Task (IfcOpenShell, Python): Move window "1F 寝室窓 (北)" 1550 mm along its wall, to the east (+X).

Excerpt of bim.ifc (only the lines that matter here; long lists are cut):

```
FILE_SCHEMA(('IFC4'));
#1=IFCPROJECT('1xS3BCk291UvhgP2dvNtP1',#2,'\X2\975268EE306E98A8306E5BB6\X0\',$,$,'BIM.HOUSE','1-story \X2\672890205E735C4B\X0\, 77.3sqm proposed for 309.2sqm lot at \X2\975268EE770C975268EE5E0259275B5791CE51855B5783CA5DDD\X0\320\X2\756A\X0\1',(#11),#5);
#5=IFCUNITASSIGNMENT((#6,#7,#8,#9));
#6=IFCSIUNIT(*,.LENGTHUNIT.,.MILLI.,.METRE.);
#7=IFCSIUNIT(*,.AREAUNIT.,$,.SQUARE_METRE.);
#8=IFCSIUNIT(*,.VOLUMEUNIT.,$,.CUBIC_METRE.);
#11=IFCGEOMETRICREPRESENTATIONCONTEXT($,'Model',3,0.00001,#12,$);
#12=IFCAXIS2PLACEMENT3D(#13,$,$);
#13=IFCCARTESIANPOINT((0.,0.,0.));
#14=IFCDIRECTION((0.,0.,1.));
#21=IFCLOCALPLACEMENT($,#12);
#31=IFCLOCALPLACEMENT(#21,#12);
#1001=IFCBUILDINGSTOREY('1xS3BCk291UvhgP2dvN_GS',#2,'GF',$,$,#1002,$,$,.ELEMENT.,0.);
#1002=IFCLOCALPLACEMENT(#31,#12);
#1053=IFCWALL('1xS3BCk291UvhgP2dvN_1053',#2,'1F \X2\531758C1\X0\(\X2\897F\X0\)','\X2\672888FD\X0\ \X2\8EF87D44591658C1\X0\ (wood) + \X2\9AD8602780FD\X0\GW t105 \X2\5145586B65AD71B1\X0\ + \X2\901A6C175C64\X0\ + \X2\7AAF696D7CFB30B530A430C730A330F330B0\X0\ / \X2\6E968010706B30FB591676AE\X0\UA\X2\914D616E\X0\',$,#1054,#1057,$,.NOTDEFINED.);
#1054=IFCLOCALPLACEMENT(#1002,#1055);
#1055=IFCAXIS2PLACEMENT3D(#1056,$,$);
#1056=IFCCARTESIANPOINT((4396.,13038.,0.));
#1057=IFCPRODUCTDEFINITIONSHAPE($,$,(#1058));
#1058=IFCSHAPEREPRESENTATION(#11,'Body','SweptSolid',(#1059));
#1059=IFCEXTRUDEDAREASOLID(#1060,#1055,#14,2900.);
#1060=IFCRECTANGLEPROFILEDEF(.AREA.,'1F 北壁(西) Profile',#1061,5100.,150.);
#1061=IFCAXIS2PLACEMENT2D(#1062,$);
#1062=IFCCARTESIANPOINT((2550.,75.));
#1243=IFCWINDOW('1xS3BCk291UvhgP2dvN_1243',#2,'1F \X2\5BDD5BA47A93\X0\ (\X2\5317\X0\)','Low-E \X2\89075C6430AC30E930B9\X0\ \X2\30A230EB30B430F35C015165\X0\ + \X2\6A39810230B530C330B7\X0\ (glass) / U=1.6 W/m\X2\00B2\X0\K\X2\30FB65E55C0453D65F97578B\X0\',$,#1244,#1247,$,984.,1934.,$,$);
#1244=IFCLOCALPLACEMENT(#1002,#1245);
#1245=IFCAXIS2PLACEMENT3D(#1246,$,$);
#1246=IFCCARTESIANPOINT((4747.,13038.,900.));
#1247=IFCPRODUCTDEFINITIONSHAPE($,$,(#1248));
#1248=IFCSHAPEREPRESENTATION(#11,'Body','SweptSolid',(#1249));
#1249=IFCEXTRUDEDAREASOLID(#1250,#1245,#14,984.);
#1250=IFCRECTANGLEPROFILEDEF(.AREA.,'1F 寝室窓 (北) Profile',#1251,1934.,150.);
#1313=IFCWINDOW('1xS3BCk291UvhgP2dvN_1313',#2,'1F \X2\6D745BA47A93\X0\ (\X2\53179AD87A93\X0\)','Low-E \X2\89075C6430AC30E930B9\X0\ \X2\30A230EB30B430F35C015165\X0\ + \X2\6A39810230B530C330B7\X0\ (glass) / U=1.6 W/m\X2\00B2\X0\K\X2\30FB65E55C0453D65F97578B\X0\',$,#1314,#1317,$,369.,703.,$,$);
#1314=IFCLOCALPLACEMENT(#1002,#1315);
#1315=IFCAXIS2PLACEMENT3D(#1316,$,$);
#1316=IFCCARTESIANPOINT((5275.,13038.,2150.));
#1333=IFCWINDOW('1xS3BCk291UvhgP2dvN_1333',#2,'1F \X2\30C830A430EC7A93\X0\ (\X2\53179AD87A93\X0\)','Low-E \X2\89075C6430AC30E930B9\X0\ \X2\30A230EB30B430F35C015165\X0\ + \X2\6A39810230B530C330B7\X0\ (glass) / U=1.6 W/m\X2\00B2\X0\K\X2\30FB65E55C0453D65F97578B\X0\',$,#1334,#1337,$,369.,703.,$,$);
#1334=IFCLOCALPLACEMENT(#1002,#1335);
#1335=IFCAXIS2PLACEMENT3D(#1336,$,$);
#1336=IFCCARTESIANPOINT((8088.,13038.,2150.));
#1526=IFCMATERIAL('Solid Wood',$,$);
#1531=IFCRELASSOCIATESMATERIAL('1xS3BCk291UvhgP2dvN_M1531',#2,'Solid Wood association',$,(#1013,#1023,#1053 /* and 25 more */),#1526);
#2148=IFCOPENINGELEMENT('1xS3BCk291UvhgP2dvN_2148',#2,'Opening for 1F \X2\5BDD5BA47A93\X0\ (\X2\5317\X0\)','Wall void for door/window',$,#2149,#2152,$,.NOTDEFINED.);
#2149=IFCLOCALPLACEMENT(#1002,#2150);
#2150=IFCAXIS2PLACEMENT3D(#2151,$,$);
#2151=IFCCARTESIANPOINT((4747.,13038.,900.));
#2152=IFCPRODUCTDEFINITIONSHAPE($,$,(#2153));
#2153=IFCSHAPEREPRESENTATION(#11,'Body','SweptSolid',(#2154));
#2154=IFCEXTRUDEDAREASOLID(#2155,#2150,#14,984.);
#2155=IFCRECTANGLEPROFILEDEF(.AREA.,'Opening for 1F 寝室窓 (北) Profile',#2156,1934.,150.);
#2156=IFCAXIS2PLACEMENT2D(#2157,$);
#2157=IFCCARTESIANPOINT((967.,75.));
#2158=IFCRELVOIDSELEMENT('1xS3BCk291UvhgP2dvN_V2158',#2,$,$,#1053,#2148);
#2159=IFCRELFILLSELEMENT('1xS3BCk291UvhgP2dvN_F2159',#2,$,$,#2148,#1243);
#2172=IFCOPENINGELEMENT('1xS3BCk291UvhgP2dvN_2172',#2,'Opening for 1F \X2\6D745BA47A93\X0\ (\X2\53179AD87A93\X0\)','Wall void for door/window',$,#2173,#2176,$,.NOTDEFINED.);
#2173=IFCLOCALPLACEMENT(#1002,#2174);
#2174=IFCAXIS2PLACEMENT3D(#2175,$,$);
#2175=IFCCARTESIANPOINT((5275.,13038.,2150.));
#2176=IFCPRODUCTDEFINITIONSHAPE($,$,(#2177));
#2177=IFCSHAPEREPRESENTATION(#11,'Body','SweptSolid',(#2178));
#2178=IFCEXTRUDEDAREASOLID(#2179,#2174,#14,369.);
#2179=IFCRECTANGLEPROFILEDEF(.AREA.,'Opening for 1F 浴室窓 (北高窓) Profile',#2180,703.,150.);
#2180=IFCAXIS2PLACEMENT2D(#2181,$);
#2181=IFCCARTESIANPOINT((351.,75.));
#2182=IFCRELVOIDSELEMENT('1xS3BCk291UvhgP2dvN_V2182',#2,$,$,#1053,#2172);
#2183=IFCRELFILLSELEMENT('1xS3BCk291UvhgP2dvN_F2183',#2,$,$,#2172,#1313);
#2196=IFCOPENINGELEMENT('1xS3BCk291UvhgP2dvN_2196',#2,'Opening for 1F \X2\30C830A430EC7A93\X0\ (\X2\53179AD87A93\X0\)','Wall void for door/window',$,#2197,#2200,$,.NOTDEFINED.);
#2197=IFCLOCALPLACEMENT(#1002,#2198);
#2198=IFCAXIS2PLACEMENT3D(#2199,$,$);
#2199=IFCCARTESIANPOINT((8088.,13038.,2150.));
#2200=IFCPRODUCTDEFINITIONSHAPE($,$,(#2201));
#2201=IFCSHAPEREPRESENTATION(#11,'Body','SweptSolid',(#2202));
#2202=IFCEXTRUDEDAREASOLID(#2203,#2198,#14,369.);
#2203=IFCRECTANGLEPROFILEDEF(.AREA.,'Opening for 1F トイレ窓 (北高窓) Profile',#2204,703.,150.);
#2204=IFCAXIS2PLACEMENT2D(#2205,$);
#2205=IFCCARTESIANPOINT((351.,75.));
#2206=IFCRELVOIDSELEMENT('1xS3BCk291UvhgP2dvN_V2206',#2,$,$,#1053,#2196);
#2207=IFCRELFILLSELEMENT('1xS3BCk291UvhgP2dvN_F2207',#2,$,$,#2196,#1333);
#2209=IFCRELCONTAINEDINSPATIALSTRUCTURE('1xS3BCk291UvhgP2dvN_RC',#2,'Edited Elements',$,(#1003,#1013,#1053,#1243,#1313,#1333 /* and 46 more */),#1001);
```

```python
import ifcopenshell
import ifcopenshell.api.geometry
import ifcopenshell.util.placement

model = ifcopenshell.open("bim.ifc")

window = model.by_id(1243)
opening = window.FillsVoids[0].RelatingOpeningElement
wall = opening.VoidsElements[0].RelatingBuildingElement

wall_matrix = ifcopenshell.util.placement.get_local_placement(wall.ObjectPlacement)
shift = wall_matrix[:3, 0] * 1550.0
before = ifcopenshell.util.placement.get_local_placement(window.ObjectPlacement)[:3, 3].copy()

# The window is not placed relative to its opening, so move both.
for product in (opening, window):
    matrix = ifcopenshell.util.placement.get_local_placement(product.ObjectPlacement)
    matrix[:3, 3] += shift
    ifcopenshell.api.geometry.edit_object_placement(model, product=product, matrix=matrix, is_si=False)

after = ifcopenshell.util.placement.get_local_placement(window.ObjectPlacement)[:3, 3]
print("window moved by", (after - before).round(3) + 0.0)

model.write("bim_rev.ifc")
```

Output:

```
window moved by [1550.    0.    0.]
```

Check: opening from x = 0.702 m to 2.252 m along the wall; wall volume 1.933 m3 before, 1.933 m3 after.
